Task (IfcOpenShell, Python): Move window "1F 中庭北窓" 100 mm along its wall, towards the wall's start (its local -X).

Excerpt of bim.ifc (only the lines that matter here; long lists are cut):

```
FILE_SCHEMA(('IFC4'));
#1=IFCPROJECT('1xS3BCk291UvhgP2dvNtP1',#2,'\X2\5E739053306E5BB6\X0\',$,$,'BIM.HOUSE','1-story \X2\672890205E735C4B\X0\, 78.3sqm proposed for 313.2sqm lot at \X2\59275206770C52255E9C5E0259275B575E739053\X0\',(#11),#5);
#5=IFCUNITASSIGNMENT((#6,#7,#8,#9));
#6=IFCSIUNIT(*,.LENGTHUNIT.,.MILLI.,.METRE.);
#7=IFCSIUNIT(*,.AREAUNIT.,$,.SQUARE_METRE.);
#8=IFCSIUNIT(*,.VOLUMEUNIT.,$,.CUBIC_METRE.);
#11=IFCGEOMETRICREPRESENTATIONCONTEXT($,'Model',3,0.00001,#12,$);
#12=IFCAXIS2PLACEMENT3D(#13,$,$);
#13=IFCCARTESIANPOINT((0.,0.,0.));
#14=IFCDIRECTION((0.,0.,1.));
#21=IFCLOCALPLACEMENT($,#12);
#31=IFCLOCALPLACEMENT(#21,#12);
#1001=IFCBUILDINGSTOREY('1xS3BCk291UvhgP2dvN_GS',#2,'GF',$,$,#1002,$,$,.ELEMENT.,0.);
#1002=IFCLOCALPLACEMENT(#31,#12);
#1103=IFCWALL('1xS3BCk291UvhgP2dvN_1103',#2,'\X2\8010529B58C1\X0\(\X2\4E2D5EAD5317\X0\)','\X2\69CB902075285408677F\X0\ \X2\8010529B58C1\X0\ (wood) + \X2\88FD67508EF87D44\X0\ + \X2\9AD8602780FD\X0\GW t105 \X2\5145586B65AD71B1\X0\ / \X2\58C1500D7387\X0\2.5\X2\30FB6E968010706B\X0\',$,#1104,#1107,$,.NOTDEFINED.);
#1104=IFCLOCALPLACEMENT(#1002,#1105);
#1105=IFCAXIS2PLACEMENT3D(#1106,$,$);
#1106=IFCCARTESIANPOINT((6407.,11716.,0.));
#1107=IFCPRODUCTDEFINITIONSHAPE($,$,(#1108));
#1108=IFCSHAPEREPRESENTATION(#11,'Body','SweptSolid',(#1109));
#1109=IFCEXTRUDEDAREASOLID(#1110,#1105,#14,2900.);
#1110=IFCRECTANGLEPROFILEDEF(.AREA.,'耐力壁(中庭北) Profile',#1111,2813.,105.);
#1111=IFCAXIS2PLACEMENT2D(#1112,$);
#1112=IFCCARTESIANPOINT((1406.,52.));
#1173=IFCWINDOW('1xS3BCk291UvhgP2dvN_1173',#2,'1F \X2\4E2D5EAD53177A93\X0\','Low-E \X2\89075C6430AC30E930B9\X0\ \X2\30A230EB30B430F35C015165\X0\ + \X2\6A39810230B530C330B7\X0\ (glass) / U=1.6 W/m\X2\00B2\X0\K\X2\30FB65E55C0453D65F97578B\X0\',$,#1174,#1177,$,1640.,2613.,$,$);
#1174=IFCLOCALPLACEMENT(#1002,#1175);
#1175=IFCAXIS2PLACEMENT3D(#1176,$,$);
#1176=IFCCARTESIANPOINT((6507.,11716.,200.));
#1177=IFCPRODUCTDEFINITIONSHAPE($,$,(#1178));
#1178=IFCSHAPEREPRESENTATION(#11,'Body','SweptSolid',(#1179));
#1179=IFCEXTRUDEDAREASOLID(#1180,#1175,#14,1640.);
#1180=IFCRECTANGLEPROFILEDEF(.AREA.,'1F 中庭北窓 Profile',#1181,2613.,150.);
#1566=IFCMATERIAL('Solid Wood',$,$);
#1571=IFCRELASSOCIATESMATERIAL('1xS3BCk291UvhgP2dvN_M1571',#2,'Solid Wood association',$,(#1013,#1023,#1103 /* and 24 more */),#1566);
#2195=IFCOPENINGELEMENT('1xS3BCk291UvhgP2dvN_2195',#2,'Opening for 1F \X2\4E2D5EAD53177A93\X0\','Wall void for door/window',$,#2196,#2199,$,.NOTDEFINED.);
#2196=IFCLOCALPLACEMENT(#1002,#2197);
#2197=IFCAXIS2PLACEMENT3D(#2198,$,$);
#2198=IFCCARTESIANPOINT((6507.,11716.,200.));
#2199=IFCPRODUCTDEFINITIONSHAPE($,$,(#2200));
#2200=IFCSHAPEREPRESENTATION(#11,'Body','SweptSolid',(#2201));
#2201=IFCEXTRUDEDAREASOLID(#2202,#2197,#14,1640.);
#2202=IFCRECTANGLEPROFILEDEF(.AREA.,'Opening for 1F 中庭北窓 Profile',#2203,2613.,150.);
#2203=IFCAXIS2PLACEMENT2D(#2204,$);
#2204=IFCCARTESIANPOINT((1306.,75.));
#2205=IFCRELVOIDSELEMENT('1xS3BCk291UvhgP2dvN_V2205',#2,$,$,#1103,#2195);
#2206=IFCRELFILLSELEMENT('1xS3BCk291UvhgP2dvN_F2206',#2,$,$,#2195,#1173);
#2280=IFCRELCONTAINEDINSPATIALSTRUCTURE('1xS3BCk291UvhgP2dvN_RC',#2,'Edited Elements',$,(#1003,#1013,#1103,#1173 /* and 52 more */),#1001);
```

```python
import ifcopenshell
import ifcopenshell.api.geometry
import ifcopenshell.util.placement

model = ifcopenshell.open("bim.ifc")

window = model.by_id(1173)
opening = window.FillsVoids[0].RelatingOpeningElement
wall = opening.VoidsElements[0].RelatingBuildingElement

wall_matrix = ifcopenshell.util.placement.get_local_placement(wall.ObjectPlacement)
shift = wall_matrix[:3, 0] * -100.0
before = ifcopenshell.util.placement.get_local_placement(window.ObjectPlacement)[:3, 3].copy()

# The window is not placed relative to its opening, so move both.
for product in (opening, window):
    matrix = ifcopenshell.util.placement.get_local_placement(product.ObjectPlacement)
    matrix[:3, 3] += shift
    ifcopenshell.api.geometry.edit_object_placement(model, product=product, matrix=matrix, is_si=False)

after = ifcopenshell.util.placement.get_local_placement(window.ObjectPlacement)[:3, 3]
print("window moved by", (after - before).round(3) + 0.0)

model.write("bim-out.ifc")
```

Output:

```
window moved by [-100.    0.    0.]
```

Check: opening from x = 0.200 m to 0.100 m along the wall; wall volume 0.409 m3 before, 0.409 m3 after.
